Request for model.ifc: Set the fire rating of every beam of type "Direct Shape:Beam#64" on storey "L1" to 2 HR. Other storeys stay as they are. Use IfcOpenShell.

First a look at what the model holds.

```python
import ifcopenshell
import ifcopenshell.util.element

model = ifcopenshell.open("model.ifc")
print(model.schema)
storey = next(s for s in model.by_type("IfcBuildingStorey") if s.Name == "L1")
beams = [e for e in ifcopenshell.util.element.get_decomposition(storey) if e.is_a("IfcBeam")]
seen = {}
for e in beams:
    element_type = ifcopenshell.util.element.get_type(e)
    key = (element_type.Name if element_type != e and element_type else None, ifcopenshell.util.element.get_pset(e, "Pset_BeamCommon", "FireRating"))
    seen[key] = seen.get(key, 0) + 1
for (name, value), count in sorted(seen.items(), key=str):
    print(count, "x", name, "|", value)
```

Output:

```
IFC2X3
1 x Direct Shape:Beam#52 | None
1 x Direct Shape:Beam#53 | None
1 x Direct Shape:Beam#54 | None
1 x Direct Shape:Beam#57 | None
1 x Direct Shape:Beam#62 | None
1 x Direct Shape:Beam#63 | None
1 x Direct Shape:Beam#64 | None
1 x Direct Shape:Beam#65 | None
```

```python
import ifcopenshell
import ifcopenshell.api.pset
import ifcopenshell.util.element

model = ifcopenshell.open("model.ifc")

storey = next(s for s in model.by_type("IfcBuildingStorey") if s.Name == "L1")
beams = [e for e in ifcopenshell.util.element.get_decomposition(storey) if e.is_a("IfcBeam")]

count = 0
for e in beams:
    element_type = ifcopenshell.util.element.get_type(e)
    if element_type in (None, e) or element_type.Name != "Direct Shape:Beam#64":
        continue
    # add_pset returns the element's existing set when there is one.
    pset = ifcopenshell.api.pset.add_pset(model, product=e, name="Pset_BeamCommon")
    ifcopenshell.api.pset.edit_pset(model, pset=pset, properties={"FireRating": "2 HR"})
    count += 1

print(count, "beams updated")

model.write("model_v2.ifc")
```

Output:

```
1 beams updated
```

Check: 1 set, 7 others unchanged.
